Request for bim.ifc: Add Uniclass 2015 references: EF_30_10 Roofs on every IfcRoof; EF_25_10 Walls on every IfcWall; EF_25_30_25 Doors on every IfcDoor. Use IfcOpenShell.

First a look at what the model holds.

```python
import ifcopenshell

model = ifcopenshell.open("bim.ifc")
print(model.schema)
print("classifications:", [c.Name for c in model.by_type("IfcClassification")])
for ifc_class in ("IfcDoor", "IfcRoof", "IfcStair", "IfcWall", "IfcWindow"):
    print(ifc_class, len(model.by_type(ifc_class)))
```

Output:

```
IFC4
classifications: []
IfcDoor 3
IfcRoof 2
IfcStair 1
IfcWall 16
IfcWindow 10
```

```python
import ifcopenshell
import ifcopenshell.api.classification

model = ifcopenshell.open("bim.ifc")

system = ifcopenshell.api.classification.add_classification(model, classification="Uniclass 2015")

codes = {
    "IfcRoof": ("EF_30_10", "Roofs"),
    "IfcWall": ("EF_25_10", "Walls"),
    "IfcDoor": ("EF_25_30_25", "Doors"),
}
for ifc_class, (code, name) in codes.items():
    products = model.by_type(ifc_class)
    ifcopenshell.api.classification.add_reference(
        model, products=products, classification=system, identification=code, name=name
    )
    print(code, len(products))

model.write("bim_edited.ifc")
```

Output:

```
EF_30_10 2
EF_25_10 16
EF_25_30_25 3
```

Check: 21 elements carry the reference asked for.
